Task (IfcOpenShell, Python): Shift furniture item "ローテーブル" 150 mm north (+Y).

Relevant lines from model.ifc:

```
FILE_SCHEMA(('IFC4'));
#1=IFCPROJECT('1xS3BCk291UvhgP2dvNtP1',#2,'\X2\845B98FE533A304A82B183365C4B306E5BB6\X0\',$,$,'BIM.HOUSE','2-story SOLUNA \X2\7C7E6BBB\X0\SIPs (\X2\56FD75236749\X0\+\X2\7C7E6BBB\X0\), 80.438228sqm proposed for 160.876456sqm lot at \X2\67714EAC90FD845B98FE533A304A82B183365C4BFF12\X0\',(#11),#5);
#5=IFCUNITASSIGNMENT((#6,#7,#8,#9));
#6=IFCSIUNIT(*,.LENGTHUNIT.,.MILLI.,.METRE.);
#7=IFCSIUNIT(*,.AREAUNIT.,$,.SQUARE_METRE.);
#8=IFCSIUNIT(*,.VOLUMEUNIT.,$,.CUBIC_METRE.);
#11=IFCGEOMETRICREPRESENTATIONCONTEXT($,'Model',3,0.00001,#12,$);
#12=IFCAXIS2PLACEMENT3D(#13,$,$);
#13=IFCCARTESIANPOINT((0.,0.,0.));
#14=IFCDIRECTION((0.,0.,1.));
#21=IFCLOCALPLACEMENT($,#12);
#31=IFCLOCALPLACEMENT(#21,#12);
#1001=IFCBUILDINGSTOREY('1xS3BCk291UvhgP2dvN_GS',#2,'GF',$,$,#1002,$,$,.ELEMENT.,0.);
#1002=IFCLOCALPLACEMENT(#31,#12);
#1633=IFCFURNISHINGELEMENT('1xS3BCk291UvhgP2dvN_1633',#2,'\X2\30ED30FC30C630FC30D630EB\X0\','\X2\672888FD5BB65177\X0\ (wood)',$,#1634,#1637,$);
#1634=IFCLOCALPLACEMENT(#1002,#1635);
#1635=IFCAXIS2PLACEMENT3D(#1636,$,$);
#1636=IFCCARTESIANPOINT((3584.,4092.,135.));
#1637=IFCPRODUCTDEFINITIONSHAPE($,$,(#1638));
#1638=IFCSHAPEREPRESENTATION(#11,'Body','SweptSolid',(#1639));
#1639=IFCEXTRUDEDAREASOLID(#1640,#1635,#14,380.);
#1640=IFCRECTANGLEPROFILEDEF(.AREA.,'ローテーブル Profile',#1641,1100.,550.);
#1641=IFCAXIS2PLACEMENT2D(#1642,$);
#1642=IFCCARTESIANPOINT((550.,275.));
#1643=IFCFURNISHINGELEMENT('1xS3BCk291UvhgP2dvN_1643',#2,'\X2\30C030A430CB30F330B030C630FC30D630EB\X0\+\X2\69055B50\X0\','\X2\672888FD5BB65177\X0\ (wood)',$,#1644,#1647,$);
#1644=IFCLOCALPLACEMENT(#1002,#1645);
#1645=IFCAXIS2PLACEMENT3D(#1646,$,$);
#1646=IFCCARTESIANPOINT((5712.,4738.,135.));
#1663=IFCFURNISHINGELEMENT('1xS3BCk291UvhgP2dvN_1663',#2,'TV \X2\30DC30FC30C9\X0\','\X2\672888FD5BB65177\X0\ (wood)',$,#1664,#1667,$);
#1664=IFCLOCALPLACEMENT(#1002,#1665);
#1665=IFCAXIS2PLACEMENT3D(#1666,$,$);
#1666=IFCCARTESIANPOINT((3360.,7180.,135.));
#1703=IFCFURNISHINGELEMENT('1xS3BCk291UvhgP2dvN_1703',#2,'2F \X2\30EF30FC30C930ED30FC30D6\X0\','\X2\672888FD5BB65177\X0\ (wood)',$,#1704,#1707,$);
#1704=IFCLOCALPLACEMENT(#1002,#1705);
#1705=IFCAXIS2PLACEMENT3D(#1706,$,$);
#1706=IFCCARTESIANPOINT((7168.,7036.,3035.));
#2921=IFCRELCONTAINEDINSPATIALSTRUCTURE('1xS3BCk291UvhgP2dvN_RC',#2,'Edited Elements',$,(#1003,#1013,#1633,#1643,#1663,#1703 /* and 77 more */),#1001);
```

```python
import ifcopenshell
import ifcopenshell.api.geometry
import ifcopenshell.util.placement
import ifcopenshell.util.unit

model = ifcopenshell.open("model.ifc")
unit_scale = ifcopenshell.util.unit.calculate_unit_scale(model)

item = model.by_guid("1xS3BCk291UvhgP2dvN_1633")
matrix = ifcopenshell.util.placement.get_local_placement(item.ObjectPlacement)
matrix[1, 3] += 0.15 / unit_scale
ifcopenshell.api.geometry.edit_object_placement(model, product=item, matrix=matrix, is_si=False)

print(ifcopenshell.util.placement.get_local_placement(item.ObjectPlacement).round(3) + 0.0)

model.write("model_updated.ifc")
```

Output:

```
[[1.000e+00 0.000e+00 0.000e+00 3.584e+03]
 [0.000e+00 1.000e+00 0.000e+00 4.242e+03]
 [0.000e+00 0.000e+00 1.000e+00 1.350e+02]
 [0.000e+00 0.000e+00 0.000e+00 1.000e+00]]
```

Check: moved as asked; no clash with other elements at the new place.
